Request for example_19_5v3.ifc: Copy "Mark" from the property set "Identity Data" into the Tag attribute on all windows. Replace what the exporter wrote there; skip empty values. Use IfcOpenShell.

First a look at what the model holds.

```python
import ifcopenshell
import ifcopenshell.util.element

model = ifcopenshell.open("example_19_5v3.ifc")
print(model.schema)
windows = model.by_type("IfcWindow")
print(len(windows), "windows")
for e in windows[:8]:
    source = ifcopenshell.util.element.get_pset(e, "Identity Data", "Mark")
    target = e.Tag
    print(e.id(), repr(source), repr(target), sep=" | ")
```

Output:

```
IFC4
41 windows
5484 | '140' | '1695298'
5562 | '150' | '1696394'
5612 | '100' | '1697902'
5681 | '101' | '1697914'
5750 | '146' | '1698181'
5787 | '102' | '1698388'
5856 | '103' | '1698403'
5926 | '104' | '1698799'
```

```python
import ifcopenshell
import ifcopenshell.util.element

model = ifcopenshell.open("example_19_5v3.ifc")

count = 0
for e in model.by_type("IfcWindow"):
    value = ifcopenshell.util.element.get_pset(e, "Identity Data", "Mark")
    current = e.Tag
    if not value or not value.strip() or current == value:
        continue
    e.Tag = value
    count += 1

print(count, "windows updated")

model.write("example_19_5v3_updated.ifc")
```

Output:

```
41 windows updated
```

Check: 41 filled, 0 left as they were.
